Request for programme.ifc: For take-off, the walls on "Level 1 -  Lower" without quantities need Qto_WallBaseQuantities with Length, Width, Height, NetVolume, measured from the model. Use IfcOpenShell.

First a look at what the model holds.

```python
import ifcopenshell
import ifcopenshell.util.element
import ifcopenshell.util.unit

model = ifcopenshell.open("programme.ifc")
print(model.schema)
for unit_type in ("LENGTHUNIT", "AREAUNIT", "VOLUMEUNIT"):
    print(unit_type, ifcopenshell.util.unit.calculate_unit_scale(model, unit_type))
storey = next(s for s in model.by_type("IfcBuildingStorey") if s.Name == "Level 1 -  Lower")
walls = [e for e in ifcopenshell.util.element.get_decomposition(storey) if e.is_a("IfcWall")]
for e in sorted(walls, key=lambda e: e.id()):
    print(e.id(), e.is_a(), e.Name, list(ifcopenshell.util.element.get_psets(e, qtos_only=True)), sep=" | ")
```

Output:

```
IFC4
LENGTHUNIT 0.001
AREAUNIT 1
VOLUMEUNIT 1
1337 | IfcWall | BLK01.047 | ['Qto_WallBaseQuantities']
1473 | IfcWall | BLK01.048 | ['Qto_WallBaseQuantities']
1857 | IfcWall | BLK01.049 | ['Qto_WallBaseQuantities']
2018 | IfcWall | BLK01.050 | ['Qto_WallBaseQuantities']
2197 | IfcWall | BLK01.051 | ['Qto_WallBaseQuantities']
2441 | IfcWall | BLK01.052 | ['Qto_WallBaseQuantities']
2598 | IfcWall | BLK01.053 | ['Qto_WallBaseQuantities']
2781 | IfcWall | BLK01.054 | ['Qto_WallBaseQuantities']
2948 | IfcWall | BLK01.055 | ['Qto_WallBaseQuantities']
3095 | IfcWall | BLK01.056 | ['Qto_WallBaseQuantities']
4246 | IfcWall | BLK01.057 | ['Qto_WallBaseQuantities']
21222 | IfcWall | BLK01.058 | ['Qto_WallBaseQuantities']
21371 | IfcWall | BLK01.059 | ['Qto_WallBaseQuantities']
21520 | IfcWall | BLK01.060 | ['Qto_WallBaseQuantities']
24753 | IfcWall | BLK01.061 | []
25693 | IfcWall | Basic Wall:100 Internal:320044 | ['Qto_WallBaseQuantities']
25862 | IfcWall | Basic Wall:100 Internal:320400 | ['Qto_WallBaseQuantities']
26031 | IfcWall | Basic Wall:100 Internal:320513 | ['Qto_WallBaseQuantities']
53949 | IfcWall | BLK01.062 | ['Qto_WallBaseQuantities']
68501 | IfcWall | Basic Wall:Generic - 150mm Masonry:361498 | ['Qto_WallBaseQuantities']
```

```python
import ifcopenshell
import ifcopenshell.api.pset
import ifcopenshell.geom
import ifcopenshell.util.element
import ifcopenshell.util.shape
import ifcopenshell.util.unit

model = ifcopenshell.open("programme.ifc")
unit_scale = ifcopenshell.util.unit.calculate_unit_scale(model)
volume_scale = ifcopenshell.util.unit.calculate_unit_scale(model, "VOLUMEUNIT")
settings = ifcopenshell.geom.settings()

storey = next(s for s in model.by_type("IfcBuildingStorey") if s.Name == "Level 1 -  Lower")
walls = [e for e in ifcopenshell.util.element.get_decomposition(storey) if e.is_a("IfcWall")]

for e in sorted(walls, key=lambda e: e.id()):
    if ifcopenshell.util.element.get_psets(e, qtos_only=True, should_inherit=False):
        continue
    # Geometry comes back in metres, in the element's own axes.
    shape = ifcopenshell.geom.create_shape(settings, e)
    values = {
        "Length": ifcopenshell.util.shape.get_x(shape.geometry) / unit_scale,
        "Width": ifcopenshell.util.shape.get_y(shape.geometry) / unit_scale,
        "Height": ifcopenshell.util.shape.get_z(shape.geometry) / unit_scale,
        "NetVolume": ifcopenshell.util.shape.get_volume(shape.geometry) / volume_scale,
    }
    qto = ifcopenshell.api.pset.add_qto(model, product=e, name="Qto_WallBaseQuantities")
    ifcopenshell.api.pset.edit_qto(model, qto=qto, properties=values)
    print(e.id(), {k: round(v, 3) for k, v in values.items()})

model.write("programme-out.ifc")
```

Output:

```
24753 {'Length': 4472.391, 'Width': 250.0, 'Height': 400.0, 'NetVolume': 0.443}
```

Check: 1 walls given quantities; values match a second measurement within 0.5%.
